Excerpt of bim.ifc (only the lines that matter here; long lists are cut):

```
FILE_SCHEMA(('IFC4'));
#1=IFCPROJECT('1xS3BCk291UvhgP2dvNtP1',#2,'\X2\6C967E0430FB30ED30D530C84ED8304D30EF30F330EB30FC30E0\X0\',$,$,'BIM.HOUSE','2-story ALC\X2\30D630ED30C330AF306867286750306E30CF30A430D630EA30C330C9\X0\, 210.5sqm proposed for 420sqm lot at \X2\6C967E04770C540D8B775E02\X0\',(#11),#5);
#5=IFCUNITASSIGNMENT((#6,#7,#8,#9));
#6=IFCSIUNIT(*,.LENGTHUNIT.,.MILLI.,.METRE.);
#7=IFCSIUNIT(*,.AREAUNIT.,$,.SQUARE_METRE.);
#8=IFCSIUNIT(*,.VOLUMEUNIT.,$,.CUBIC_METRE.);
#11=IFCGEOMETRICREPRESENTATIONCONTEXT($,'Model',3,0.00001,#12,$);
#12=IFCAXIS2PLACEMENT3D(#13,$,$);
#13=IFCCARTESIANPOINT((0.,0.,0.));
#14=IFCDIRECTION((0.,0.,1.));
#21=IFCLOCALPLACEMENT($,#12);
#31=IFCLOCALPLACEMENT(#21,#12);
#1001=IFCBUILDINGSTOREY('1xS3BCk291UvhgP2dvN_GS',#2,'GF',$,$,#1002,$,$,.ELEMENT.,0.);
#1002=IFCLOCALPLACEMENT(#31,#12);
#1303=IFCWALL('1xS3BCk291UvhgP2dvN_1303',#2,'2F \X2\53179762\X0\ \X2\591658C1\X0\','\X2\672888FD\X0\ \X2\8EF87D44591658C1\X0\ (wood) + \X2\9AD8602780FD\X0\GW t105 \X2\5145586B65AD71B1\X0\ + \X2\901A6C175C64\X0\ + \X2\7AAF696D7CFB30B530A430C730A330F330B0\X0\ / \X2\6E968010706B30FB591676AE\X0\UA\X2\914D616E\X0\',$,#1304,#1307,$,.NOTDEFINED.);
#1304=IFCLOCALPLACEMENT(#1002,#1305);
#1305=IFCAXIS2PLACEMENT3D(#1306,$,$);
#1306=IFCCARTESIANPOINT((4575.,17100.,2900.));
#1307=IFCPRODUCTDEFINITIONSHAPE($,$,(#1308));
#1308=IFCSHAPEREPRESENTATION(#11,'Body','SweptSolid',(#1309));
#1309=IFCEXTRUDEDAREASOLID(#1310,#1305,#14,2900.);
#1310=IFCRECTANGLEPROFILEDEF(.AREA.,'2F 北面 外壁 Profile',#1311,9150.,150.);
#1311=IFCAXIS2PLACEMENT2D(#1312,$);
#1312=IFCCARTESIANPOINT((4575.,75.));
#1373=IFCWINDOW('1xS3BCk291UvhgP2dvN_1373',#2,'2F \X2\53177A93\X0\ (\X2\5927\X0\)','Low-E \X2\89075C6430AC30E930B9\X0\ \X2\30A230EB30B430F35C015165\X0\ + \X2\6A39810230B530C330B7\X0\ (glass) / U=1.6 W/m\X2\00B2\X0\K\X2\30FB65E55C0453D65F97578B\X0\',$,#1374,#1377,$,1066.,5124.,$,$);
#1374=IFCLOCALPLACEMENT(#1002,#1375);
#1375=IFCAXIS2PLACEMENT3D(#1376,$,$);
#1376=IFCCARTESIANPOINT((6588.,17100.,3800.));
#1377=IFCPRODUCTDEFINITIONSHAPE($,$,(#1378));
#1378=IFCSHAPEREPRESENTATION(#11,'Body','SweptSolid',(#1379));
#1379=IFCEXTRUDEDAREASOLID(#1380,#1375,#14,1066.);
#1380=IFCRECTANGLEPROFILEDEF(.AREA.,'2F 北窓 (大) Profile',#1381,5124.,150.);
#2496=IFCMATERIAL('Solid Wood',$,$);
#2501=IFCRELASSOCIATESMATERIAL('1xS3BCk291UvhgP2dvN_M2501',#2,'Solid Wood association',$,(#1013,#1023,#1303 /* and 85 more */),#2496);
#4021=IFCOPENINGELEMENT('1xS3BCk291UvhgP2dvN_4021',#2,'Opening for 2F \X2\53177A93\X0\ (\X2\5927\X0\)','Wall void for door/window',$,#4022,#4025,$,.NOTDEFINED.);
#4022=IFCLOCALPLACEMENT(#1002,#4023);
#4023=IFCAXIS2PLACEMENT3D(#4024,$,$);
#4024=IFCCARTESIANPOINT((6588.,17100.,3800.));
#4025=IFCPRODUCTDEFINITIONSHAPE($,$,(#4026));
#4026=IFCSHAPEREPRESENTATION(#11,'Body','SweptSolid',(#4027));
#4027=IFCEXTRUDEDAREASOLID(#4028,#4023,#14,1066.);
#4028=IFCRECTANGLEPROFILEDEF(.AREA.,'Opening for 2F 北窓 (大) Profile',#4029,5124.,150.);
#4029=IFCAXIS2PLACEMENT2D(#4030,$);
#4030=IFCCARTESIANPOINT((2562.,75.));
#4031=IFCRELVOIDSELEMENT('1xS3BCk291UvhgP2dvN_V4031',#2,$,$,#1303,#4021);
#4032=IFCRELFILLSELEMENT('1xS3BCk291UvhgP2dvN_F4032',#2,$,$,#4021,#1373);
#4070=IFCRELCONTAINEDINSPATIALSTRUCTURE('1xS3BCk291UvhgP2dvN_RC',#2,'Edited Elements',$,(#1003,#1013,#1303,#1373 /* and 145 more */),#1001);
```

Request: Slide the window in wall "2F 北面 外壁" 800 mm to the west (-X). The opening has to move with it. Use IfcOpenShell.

```python
import ifcopenshell
import ifcopenshell.api.geometry
import ifcopenshell.util.placement
import ifcopenshell.util.unit

model = ifcopenshell.open("bim.ifc")
unit_scale = ifcopenshell.util.unit.calculate_unit_scale(model)

window = model.by_guid("1xS3BCk291UvhgP2dvN_1373")
opening = window.FillsVoids[0].RelatingOpeningElement
wall = opening.VoidsElements[0].RelatingBuildingElement

wall_matrix = ifcopenshell.util.placement.get_local_placement(wall.ObjectPlacement)
shift = wall_matrix[:3, 0] * -0.8 / unit_scale
before = ifcopenshell.util.placement.get_local_placement(window.ObjectPlacement)[:3, 3].copy()

# The window is not placed relative to its opening, so move both.
for product in (opening, window):
    matrix = ifcopenshell.util.placement.get_local_placement(product.ObjectPlacement)
    matrix[:3, 3] += shift
    ifcopenshell.api.geometry.edit_object_placement(model, product=product, matrix=matrix, is_si=False)

after = ifcopenshell.util.placement.get_local_placement(window.ObjectPlacement)[:3, 3]
print("window moved by", (after - before).round(3) + 0.0)

model.write("bim_v2.ifc")
```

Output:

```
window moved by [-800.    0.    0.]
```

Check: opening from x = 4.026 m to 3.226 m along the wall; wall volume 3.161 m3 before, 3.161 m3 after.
